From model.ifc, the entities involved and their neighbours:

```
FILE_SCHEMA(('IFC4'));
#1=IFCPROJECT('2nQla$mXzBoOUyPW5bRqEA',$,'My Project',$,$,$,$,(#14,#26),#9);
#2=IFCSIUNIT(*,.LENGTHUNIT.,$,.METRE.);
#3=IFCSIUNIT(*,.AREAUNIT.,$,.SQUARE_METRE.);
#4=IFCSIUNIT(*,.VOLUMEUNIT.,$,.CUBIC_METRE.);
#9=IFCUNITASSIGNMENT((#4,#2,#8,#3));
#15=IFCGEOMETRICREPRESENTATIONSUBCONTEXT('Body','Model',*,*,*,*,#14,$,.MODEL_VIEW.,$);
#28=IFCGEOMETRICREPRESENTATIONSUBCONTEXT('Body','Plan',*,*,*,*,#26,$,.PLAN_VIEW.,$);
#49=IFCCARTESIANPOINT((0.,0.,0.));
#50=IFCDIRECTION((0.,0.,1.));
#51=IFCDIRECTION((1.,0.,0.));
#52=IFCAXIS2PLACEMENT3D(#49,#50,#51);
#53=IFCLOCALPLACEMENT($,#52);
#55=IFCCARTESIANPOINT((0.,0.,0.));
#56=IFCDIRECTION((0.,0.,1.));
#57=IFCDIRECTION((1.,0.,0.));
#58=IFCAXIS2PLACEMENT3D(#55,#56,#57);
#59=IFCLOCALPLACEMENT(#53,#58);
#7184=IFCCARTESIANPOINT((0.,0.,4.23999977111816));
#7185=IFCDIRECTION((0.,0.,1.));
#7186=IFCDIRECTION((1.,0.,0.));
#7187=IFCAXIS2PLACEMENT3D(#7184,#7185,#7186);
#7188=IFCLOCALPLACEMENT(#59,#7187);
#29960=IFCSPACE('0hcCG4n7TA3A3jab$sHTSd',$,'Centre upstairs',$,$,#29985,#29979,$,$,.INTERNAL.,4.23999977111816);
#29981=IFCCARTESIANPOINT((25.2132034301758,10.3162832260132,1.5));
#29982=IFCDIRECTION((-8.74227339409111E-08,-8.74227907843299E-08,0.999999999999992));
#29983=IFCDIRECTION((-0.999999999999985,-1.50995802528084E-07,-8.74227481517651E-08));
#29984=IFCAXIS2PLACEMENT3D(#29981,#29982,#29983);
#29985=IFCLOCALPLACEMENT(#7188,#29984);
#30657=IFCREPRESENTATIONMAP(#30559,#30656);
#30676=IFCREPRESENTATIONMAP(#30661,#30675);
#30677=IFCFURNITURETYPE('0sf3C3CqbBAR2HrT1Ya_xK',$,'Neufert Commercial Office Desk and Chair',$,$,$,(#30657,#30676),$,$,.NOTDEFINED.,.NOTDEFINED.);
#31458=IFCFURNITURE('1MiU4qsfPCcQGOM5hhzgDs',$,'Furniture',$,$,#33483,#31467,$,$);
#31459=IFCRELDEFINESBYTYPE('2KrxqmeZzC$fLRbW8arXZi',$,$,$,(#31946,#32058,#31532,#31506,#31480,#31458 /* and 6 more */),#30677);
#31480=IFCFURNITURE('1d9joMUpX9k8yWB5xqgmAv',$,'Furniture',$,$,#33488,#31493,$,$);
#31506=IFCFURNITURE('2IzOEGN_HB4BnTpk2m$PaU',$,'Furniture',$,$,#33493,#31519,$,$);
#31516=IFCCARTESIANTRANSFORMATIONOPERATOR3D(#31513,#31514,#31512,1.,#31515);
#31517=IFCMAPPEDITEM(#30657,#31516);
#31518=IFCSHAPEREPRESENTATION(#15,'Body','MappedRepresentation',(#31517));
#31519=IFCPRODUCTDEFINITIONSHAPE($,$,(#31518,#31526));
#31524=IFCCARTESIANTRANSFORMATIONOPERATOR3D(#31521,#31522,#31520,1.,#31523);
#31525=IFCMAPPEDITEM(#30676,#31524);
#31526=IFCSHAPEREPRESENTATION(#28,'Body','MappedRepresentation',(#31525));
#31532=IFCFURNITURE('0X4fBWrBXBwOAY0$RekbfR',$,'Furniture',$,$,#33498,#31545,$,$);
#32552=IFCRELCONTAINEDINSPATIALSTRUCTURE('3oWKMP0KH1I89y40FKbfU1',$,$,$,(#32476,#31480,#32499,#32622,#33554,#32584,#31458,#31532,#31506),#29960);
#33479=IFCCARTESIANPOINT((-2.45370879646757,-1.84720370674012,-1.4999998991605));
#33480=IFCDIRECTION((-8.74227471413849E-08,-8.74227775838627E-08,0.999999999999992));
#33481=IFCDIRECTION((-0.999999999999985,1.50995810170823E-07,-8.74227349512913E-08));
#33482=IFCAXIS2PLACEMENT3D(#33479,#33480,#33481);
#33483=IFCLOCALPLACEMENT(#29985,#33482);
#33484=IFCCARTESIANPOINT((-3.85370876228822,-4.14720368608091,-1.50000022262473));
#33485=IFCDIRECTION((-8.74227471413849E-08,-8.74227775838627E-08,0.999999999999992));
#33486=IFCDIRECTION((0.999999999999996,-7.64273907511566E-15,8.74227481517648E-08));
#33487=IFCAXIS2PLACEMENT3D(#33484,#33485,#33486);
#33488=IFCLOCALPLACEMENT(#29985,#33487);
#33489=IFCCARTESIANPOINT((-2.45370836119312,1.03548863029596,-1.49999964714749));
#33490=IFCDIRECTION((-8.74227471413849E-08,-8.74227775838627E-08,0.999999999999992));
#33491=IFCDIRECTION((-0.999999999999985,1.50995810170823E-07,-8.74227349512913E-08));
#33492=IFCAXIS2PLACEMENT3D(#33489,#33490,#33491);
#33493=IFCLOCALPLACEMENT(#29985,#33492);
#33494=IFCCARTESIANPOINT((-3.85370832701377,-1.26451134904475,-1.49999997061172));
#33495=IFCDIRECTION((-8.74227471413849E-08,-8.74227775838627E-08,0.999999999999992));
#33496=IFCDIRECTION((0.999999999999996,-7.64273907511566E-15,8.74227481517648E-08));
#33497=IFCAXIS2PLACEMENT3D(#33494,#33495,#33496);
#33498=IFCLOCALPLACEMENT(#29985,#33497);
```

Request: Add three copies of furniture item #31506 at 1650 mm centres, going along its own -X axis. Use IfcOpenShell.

```python
import ifcopenshell
import ifcopenshell.api.geometry
import ifcopenshell.api.root
import ifcopenshell.util.element
import ifcopenshell.util.placement

model = ifcopenshell.open("model.ifc")

source = model.by_guid("2IzOEGN_HB4BnTpk2m$PaU")
base = ifcopenshell.util.placement.get_local_placement(source.ObjectPlacement)
step = -base[:3, 0] * 1.65

for i in range(1, 4):
    copy = ifcopenshell.api.root.copy_class(model, product=source)
    copy.Representation = ifcopenshell.util.element.copy_deep(
        model, source.Representation, exclude=["IfcGeometricRepresentationContext", "IfcRepresentationMap"]
    )
    matrix = base.copy()
    matrix[:3, 3] += i * step
    print("added at", matrix[:3, 3].round(3) + 0.0)
    ifcopenshell.api.geometry.edit_object_placement(model, product=copy, matrix=matrix, is_si=False)

model.write("model-out.ifc")
```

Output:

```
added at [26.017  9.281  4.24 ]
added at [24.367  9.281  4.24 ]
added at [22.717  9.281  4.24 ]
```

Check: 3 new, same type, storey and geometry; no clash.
